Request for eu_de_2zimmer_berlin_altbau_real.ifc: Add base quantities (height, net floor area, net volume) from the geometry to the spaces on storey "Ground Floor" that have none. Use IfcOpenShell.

First a look at what the model holds.

```python
import ifcopenshell
import ifcopenshell.util.element
import ifcopenshell.util.unit

model = ifcopenshell.open("eu_de_2zimmer_berlin_altbau_real.ifc")
print(model.schema)
for unit_type in ("LENGTHUNIT", "AREAUNIT", "VOLUMEUNIT"):
    print(unit_type, ifcopenshell.util.unit.calculate_unit_scale(model, unit_type))
storey = next(s for s in model.by_type("IfcBuildingStorey") if s.Name == "Ground Floor")
spaces = [e for e in ifcopenshell.util.element.get_decomposition(storey) if e.is_a("IfcSpace")]
for e in sorted(spaces, key=lambda e: e.id()):
    print(e.id(), e.is_a(), e.Name, list(ifcopenshell.util.element.get_psets(e, qtos_only=True)), sep=" | ")
```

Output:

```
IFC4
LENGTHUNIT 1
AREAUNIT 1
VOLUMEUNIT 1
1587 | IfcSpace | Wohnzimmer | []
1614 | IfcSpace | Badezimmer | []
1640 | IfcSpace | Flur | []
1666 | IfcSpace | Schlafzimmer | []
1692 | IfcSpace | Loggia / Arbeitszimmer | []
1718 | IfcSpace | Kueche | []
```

```python
import ifcopenshell
import ifcopenshell.api.pset
import ifcopenshell.geom
import ifcopenshell.util.element
import ifcopenshell.util.shape
import ifcopenshell.util.unit

model = ifcopenshell.open("eu_de_2zimmer_berlin_altbau_real.ifc")
unit_scale = ifcopenshell.util.unit.calculate_unit_scale(model)
area_scale = ifcopenshell.util.unit.calculate_unit_scale(model, "AREAUNIT")
volume_scale = ifcopenshell.util.unit.calculate_unit_scale(model, "VOLUMEUNIT")
settings = ifcopenshell.geom.settings()

storey = next(s for s in model.by_type("IfcBuildingStorey") if s.Name == "Ground Floor")
spaces = [e for e in ifcopenshell.util.element.get_decomposition(storey) if e.is_a("IfcSpace")]

for e in sorted(spaces, key=lambda e: e.id()):
    if ifcopenshell.util.element.get_psets(e, qtos_only=True, should_inherit=False):
        continue
    # Geometry comes back in metres, in the element's own axes.
    shape = ifcopenshell.geom.create_shape(settings, e)
    values = {
        "Height": ifcopenshell.util.shape.get_z(shape.geometry) / unit_scale,
        "NetFloorArea": ifcopenshell.util.shape.get_footprint_area(shape.geometry) / area_scale,
        "NetVolume": ifcopenshell.util.shape.get_volume(shape.geometry) / volume_scale,
    }
    qto = ifcopenshell.api.pset.add_qto(model, product=e, name="Qto_SpaceBaseQuantities")
    ifcopenshell.api.pset.edit_qto(model, qto=qto, properties=values)
    print(e.id(), {k: round(v, 3) for k, v in values.items()})

model.write("eu_de_2zimmer_berlin_altbau_real_updated.ifc")
```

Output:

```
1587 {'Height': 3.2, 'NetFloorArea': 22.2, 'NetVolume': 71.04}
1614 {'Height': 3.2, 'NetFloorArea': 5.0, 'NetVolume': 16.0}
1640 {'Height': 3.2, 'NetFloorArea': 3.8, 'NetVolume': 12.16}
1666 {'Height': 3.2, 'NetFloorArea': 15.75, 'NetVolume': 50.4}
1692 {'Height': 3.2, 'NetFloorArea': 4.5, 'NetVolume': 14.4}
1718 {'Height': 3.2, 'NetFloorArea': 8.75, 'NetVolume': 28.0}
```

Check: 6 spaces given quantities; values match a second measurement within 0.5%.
